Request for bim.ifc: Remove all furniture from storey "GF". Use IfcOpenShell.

First a look at what the model holds.

```python
import ifcopenshell
import ifcopenshell.util.element

model = ifcopenshell.open("bim.ifc")
print(model.schema)
storey = next(s for s in model.by_type("IfcBuildingStorey") if s.Name == "GF")
furniture = [e for e in ifcopenshell.util.element.get_decomposition(storey) if e.is_a("IfcFurnishingElement")]
seen = {}
for e in furniture:
    element_type = ifcopenshell.util.element.get_type(e)
    name = element_type.Name if element_type not in (None, e) else None
    seen[name] = seen.get(name, 0) + 1
for name, count in sorted(seen.items(), key=str):
    print(count, "x", name)
```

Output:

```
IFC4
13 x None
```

```python
import ifcopenshell
import ifcopenshell.api.root
import ifcopenshell.util.element

model = ifcopenshell.open("bim.ifc")

storey = next(s for s in model.by_type("IfcBuildingStorey") if s.Name == "GF")
furniture = [e for e in ifcopenshell.util.element.get_decomposition(storey) if e.is_a("IfcFurnishingElement")]

for e in furniture:
    ifcopenshell.api.root.remove_product(model, product=e)
print(len(furniture), "removed")

model.write("bim-out.ifc")
```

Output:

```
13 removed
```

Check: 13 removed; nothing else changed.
